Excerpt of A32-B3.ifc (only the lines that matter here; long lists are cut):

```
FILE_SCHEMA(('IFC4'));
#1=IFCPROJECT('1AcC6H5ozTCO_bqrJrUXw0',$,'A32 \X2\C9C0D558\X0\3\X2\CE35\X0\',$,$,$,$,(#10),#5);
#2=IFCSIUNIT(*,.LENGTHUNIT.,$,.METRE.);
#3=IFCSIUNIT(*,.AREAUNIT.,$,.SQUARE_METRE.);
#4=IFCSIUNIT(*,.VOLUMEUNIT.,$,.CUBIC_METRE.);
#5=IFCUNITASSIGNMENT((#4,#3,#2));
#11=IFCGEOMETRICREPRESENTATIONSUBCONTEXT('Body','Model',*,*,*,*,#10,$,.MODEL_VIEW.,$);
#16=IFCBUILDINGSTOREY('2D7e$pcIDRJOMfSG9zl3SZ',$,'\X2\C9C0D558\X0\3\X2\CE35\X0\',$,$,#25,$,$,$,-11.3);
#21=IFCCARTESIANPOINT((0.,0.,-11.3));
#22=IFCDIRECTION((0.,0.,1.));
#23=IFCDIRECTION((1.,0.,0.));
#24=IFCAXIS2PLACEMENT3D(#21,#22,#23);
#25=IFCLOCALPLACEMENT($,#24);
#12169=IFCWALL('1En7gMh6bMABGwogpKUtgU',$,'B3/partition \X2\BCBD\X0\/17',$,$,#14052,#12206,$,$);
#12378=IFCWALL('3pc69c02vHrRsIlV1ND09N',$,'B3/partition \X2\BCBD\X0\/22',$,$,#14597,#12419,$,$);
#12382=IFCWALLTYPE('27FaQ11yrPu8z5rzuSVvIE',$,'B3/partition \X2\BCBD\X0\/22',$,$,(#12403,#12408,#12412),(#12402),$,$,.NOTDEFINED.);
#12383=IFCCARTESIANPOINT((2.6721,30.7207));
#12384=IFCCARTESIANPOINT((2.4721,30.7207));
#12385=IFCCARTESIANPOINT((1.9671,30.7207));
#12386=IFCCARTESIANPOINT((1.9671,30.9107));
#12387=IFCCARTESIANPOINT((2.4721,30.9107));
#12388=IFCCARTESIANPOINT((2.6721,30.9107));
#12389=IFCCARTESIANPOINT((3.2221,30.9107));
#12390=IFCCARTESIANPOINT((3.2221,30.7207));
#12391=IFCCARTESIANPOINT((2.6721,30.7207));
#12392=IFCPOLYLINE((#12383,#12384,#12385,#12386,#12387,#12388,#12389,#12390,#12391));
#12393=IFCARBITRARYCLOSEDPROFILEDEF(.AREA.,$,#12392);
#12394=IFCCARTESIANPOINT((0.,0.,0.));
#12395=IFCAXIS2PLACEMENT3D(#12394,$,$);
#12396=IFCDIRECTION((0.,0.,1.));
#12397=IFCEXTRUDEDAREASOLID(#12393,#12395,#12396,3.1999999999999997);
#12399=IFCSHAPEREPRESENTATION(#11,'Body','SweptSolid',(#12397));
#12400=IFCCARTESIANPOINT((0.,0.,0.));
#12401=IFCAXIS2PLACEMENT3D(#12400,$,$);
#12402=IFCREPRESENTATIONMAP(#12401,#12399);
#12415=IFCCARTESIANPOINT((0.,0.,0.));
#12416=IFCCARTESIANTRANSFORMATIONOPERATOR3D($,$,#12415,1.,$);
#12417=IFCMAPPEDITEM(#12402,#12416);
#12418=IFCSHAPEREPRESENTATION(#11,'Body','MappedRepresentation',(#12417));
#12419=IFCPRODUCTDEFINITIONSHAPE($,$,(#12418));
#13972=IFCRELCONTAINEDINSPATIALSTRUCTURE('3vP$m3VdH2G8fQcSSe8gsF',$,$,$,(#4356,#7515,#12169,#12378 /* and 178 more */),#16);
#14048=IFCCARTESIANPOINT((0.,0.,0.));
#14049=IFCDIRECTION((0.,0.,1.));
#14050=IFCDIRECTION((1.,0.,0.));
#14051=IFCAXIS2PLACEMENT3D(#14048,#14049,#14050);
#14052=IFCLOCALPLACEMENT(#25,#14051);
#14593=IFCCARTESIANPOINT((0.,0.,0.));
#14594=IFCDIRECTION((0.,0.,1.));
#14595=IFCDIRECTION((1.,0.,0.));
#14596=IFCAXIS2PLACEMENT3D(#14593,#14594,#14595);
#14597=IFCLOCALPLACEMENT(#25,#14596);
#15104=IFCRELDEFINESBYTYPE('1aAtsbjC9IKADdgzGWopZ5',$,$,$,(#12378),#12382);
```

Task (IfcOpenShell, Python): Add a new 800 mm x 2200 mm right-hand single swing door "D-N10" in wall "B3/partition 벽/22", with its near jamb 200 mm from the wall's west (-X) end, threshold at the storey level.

```python
import numpy as np
import ifcopenshell
import ifcopenshell.api.feature
import ifcopenshell.api.geometry
import ifcopenshell.api.root
import ifcopenshell.api.spatial
import ifcopenshell.geom
import ifcopenshell.util.element
import ifcopenshell.util.placement
import ifcopenshell.util.representation
import ifcopenshell.util.shape
import ifcopenshell.util.unit

model = ifcopenshell.open("A32-B3.ifc")
unit_scale = ifcopenshell.util.unit.calculate_unit_scale(model)
settings = ifcopenshell.geom.settings()


def volume(element):
    """Net volume in cubic metres, openings subtracted."""
    shape = ifcopenshell.geom.create_shape(settings, element)
    return ifcopenshell.util.shape.get_volume(shape.geometry)


wall = model.by_id(12378)
storey = ifcopenshell.util.element.get_container(wall, ifc_class="IfcBuildingStorey")
context = ifcopenshell.util.representation.get_context(model, "Model", "Body", "MODEL_VIEW")
before = volume(wall)

width, height, from_end, sill = 0.8, 2.2, 0.2, 0.0  # metres

# The wall runs along its own X axis, and the end named is its -X end.
wall_shape = ifcopenshell.geom.create_shape(settings, wall)
x, y, z = ifcopenshell.util.shape.get_vertices(wall_shape.geometry).T
start = x.min() + from_end
face, thickness = float(y.min()), float(y.max() - y.min())
wall_matrix = ifcopenshell.util.placement.get_local_placement(wall.ObjectPlacement)
level = ifcopenshell.util.placement.get_local_placement(storey.ObjectPlacement)[2, 3]


def in_wall(x, y):
    """Placement at x, y metres in the wall's axes, at sill height."""
    matrix = wall_matrix.copy()
    matrix[:, 3] = wall_matrix @ np.array([x / unit_scale, y / unit_scale, 0.0, 1.0])
    matrix[2, 3] = level + sill / unit_scale
    return matrix


# Opening: a box that overshoots both wall faces by 50 mm.
opening = ifcopenshell.api.root.create_entity(model, ifc_class="IfcOpeningElement", predefined_type="OPENING")
box = ifcopenshell.api.geometry.add_wall_representation(
    model, context=context, length=width, height=height, thickness=thickness + 0.1
)
ifcopenshell.api.geometry.assign_representation(model, product=opening, representation=box)
ifcopenshell.api.geometry.edit_object_placement(model, product=opening, matrix=in_wall(start, face - 0.05), is_si=False)
ifcopenshell.api.feature.add_feature(model, feature=opening, element=wall)

door = ifcopenshell.api.root.create_entity(model, ifc_class="IfcDoor", name="D-N10", predefined_type="DOOR")
door.OverallWidth, door.OverallHeight = width / unit_scale, height / unit_scale
door.OperationType = "SINGLE_SWING_RIGHT"
body = ifcopenshell.api.geometry.add_door_representation(
    model,
    context=context,
    overall_width=door.OverallWidth,
    overall_height=door.OverallHeight,
    operation_type="SINGLE_SWING_RIGHT",
    lining_properties={"LiningDepth": thickness / unit_scale, "ThresholdDepth": thickness / unit_scale},
)
ifcopenshell.api.geometry.assign_representation(model, product=door, representation=body)
ifcopenshell.api.spatial.assign_container(model, products=[door], relating_structure=storey)
ifcopenshell.api.feature.add_filling(model, opening=opening, element=door)

# The lining spans the wall, so the door starts at the wall face.
ifcopenshell.api.geometry.edit_object_placement(model, product=door, matrix=in_wall(start, face), is_si=False)

after = volume(wall)

print(f"wall volume {before:.3f} -> {after:.3f} m3")

model.write("A32-B3_rev.ifc")
```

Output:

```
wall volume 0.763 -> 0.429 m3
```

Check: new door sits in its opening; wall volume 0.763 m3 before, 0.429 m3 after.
